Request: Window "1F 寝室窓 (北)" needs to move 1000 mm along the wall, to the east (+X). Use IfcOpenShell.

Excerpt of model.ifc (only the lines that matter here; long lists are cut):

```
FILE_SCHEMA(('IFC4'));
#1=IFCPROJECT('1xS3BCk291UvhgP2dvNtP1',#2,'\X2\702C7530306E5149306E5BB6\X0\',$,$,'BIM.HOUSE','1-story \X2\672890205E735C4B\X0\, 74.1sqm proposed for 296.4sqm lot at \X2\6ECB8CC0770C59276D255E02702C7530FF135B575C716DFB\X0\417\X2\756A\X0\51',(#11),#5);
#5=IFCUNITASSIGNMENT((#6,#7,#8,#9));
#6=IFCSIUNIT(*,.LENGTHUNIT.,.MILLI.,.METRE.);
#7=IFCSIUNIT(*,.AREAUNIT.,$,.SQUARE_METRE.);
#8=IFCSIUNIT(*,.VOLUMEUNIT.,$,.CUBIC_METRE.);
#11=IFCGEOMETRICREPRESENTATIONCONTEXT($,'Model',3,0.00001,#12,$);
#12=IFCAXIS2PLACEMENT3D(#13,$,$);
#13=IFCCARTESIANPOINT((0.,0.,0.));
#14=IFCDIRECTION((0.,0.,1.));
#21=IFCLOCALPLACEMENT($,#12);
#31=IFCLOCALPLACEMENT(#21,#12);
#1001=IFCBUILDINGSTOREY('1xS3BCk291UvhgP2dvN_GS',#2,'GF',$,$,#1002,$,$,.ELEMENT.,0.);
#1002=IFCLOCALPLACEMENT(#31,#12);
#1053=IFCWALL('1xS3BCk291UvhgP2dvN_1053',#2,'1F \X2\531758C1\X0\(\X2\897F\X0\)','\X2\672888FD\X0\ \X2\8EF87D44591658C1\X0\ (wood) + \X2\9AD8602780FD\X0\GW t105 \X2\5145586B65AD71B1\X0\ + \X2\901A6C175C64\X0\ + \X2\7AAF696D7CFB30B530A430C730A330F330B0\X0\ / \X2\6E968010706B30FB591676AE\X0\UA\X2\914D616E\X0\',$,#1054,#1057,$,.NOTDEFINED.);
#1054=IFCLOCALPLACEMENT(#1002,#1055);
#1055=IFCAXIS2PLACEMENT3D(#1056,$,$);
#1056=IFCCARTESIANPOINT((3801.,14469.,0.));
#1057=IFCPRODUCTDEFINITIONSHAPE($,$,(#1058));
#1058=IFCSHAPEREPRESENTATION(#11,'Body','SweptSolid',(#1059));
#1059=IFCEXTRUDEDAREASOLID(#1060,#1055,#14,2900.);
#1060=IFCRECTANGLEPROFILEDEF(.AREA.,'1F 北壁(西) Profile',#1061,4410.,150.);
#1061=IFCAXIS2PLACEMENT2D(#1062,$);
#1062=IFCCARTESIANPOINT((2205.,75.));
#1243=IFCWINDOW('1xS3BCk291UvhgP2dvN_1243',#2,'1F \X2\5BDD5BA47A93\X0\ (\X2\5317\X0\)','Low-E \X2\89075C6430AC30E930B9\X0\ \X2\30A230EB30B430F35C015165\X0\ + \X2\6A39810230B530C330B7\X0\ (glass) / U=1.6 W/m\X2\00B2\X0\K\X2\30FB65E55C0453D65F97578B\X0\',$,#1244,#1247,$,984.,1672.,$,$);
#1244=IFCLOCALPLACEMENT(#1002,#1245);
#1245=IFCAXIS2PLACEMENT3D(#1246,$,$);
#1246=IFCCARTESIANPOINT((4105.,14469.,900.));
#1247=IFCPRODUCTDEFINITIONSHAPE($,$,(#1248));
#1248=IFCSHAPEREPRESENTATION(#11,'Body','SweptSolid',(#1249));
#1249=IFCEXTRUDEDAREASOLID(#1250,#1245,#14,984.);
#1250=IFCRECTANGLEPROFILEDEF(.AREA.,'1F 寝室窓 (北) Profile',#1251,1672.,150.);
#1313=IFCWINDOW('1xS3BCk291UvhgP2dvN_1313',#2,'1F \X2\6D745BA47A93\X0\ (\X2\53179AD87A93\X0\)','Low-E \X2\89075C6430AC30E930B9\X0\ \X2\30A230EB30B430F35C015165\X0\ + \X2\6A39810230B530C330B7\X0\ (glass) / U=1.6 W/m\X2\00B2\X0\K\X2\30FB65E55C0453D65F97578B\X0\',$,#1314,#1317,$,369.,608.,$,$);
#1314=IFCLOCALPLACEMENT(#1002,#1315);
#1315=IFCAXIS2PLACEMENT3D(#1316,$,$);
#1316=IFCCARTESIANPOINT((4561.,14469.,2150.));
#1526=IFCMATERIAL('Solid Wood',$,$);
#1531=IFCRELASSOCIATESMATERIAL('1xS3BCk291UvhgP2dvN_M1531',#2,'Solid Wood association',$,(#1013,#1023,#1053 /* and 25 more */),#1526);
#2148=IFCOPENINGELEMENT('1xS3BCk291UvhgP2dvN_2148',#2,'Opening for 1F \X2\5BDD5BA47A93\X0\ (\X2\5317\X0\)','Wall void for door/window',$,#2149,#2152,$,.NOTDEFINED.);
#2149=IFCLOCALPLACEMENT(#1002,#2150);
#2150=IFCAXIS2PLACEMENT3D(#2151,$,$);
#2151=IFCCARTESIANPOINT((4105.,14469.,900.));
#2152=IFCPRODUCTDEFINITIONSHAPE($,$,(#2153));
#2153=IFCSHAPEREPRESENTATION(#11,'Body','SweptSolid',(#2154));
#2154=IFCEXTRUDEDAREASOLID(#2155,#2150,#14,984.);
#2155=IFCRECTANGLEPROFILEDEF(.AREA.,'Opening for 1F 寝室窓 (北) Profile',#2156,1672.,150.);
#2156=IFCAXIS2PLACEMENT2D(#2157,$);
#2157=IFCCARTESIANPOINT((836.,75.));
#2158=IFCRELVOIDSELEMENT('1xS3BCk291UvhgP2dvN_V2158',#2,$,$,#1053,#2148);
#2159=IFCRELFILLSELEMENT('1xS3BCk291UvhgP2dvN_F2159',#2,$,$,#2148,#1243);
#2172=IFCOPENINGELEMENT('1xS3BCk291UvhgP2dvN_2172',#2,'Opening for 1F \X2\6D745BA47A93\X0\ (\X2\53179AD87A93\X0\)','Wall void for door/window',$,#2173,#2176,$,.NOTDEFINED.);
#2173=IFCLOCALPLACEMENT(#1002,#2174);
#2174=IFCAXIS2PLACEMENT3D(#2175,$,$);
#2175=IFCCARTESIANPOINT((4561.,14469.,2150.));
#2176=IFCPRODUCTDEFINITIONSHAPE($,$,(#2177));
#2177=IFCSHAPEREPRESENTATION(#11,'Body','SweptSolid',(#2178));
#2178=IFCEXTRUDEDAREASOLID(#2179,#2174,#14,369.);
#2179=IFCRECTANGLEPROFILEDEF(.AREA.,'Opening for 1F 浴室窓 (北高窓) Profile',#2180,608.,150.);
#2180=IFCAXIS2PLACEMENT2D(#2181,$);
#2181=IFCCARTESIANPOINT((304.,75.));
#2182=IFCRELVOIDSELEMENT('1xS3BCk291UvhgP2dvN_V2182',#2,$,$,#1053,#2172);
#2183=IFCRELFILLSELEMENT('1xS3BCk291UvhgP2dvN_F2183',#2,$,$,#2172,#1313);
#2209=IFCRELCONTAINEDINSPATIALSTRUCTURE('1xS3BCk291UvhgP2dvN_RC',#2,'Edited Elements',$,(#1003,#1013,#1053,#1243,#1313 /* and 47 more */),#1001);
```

```python
import ifcopenshell
import ifcopenshell.api.geometry
import ifcopenshell.util.placement

model = ifcopenshell.open("model.ifc")

window = model.by_guid("1xS3BCk291UvhgP2dvN_1243")
opening = window.FillsVoids[0].RelatingOpeningElement
wall = opening.VoidsElements[0].RelatingBuildingElement

wall_matrix = ifcopenshell.util.placement.get_local_placement(wall.ObjectPlacement)
shift = wall_matrix[:3, 0] * 1000.0
before = ifcopenshell.util.placement.get_local_placement(window.ObjectPlacement)[:3, 3].copy()

# The window is not placed relative to its opening, so move both.
for product in (opening, window):
    matrix = ifcopenshell.util.placement.get_local_placement(product.ObjectPlacement)
    matrix[:3, 3] += shift
    ifcopenshell.api.geometry.edit_object_placement(model, product=product, matrix=matrix, is_si=False)

after = ifcopenshell.util.placement.get_local_placement(window.ObjectPlacement)[:3, 3]
print("window moved by", (after - before).round(3) + 0.0)

model.write("model-out.ifc")
```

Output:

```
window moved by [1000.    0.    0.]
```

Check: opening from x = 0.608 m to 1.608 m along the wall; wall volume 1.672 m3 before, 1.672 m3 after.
